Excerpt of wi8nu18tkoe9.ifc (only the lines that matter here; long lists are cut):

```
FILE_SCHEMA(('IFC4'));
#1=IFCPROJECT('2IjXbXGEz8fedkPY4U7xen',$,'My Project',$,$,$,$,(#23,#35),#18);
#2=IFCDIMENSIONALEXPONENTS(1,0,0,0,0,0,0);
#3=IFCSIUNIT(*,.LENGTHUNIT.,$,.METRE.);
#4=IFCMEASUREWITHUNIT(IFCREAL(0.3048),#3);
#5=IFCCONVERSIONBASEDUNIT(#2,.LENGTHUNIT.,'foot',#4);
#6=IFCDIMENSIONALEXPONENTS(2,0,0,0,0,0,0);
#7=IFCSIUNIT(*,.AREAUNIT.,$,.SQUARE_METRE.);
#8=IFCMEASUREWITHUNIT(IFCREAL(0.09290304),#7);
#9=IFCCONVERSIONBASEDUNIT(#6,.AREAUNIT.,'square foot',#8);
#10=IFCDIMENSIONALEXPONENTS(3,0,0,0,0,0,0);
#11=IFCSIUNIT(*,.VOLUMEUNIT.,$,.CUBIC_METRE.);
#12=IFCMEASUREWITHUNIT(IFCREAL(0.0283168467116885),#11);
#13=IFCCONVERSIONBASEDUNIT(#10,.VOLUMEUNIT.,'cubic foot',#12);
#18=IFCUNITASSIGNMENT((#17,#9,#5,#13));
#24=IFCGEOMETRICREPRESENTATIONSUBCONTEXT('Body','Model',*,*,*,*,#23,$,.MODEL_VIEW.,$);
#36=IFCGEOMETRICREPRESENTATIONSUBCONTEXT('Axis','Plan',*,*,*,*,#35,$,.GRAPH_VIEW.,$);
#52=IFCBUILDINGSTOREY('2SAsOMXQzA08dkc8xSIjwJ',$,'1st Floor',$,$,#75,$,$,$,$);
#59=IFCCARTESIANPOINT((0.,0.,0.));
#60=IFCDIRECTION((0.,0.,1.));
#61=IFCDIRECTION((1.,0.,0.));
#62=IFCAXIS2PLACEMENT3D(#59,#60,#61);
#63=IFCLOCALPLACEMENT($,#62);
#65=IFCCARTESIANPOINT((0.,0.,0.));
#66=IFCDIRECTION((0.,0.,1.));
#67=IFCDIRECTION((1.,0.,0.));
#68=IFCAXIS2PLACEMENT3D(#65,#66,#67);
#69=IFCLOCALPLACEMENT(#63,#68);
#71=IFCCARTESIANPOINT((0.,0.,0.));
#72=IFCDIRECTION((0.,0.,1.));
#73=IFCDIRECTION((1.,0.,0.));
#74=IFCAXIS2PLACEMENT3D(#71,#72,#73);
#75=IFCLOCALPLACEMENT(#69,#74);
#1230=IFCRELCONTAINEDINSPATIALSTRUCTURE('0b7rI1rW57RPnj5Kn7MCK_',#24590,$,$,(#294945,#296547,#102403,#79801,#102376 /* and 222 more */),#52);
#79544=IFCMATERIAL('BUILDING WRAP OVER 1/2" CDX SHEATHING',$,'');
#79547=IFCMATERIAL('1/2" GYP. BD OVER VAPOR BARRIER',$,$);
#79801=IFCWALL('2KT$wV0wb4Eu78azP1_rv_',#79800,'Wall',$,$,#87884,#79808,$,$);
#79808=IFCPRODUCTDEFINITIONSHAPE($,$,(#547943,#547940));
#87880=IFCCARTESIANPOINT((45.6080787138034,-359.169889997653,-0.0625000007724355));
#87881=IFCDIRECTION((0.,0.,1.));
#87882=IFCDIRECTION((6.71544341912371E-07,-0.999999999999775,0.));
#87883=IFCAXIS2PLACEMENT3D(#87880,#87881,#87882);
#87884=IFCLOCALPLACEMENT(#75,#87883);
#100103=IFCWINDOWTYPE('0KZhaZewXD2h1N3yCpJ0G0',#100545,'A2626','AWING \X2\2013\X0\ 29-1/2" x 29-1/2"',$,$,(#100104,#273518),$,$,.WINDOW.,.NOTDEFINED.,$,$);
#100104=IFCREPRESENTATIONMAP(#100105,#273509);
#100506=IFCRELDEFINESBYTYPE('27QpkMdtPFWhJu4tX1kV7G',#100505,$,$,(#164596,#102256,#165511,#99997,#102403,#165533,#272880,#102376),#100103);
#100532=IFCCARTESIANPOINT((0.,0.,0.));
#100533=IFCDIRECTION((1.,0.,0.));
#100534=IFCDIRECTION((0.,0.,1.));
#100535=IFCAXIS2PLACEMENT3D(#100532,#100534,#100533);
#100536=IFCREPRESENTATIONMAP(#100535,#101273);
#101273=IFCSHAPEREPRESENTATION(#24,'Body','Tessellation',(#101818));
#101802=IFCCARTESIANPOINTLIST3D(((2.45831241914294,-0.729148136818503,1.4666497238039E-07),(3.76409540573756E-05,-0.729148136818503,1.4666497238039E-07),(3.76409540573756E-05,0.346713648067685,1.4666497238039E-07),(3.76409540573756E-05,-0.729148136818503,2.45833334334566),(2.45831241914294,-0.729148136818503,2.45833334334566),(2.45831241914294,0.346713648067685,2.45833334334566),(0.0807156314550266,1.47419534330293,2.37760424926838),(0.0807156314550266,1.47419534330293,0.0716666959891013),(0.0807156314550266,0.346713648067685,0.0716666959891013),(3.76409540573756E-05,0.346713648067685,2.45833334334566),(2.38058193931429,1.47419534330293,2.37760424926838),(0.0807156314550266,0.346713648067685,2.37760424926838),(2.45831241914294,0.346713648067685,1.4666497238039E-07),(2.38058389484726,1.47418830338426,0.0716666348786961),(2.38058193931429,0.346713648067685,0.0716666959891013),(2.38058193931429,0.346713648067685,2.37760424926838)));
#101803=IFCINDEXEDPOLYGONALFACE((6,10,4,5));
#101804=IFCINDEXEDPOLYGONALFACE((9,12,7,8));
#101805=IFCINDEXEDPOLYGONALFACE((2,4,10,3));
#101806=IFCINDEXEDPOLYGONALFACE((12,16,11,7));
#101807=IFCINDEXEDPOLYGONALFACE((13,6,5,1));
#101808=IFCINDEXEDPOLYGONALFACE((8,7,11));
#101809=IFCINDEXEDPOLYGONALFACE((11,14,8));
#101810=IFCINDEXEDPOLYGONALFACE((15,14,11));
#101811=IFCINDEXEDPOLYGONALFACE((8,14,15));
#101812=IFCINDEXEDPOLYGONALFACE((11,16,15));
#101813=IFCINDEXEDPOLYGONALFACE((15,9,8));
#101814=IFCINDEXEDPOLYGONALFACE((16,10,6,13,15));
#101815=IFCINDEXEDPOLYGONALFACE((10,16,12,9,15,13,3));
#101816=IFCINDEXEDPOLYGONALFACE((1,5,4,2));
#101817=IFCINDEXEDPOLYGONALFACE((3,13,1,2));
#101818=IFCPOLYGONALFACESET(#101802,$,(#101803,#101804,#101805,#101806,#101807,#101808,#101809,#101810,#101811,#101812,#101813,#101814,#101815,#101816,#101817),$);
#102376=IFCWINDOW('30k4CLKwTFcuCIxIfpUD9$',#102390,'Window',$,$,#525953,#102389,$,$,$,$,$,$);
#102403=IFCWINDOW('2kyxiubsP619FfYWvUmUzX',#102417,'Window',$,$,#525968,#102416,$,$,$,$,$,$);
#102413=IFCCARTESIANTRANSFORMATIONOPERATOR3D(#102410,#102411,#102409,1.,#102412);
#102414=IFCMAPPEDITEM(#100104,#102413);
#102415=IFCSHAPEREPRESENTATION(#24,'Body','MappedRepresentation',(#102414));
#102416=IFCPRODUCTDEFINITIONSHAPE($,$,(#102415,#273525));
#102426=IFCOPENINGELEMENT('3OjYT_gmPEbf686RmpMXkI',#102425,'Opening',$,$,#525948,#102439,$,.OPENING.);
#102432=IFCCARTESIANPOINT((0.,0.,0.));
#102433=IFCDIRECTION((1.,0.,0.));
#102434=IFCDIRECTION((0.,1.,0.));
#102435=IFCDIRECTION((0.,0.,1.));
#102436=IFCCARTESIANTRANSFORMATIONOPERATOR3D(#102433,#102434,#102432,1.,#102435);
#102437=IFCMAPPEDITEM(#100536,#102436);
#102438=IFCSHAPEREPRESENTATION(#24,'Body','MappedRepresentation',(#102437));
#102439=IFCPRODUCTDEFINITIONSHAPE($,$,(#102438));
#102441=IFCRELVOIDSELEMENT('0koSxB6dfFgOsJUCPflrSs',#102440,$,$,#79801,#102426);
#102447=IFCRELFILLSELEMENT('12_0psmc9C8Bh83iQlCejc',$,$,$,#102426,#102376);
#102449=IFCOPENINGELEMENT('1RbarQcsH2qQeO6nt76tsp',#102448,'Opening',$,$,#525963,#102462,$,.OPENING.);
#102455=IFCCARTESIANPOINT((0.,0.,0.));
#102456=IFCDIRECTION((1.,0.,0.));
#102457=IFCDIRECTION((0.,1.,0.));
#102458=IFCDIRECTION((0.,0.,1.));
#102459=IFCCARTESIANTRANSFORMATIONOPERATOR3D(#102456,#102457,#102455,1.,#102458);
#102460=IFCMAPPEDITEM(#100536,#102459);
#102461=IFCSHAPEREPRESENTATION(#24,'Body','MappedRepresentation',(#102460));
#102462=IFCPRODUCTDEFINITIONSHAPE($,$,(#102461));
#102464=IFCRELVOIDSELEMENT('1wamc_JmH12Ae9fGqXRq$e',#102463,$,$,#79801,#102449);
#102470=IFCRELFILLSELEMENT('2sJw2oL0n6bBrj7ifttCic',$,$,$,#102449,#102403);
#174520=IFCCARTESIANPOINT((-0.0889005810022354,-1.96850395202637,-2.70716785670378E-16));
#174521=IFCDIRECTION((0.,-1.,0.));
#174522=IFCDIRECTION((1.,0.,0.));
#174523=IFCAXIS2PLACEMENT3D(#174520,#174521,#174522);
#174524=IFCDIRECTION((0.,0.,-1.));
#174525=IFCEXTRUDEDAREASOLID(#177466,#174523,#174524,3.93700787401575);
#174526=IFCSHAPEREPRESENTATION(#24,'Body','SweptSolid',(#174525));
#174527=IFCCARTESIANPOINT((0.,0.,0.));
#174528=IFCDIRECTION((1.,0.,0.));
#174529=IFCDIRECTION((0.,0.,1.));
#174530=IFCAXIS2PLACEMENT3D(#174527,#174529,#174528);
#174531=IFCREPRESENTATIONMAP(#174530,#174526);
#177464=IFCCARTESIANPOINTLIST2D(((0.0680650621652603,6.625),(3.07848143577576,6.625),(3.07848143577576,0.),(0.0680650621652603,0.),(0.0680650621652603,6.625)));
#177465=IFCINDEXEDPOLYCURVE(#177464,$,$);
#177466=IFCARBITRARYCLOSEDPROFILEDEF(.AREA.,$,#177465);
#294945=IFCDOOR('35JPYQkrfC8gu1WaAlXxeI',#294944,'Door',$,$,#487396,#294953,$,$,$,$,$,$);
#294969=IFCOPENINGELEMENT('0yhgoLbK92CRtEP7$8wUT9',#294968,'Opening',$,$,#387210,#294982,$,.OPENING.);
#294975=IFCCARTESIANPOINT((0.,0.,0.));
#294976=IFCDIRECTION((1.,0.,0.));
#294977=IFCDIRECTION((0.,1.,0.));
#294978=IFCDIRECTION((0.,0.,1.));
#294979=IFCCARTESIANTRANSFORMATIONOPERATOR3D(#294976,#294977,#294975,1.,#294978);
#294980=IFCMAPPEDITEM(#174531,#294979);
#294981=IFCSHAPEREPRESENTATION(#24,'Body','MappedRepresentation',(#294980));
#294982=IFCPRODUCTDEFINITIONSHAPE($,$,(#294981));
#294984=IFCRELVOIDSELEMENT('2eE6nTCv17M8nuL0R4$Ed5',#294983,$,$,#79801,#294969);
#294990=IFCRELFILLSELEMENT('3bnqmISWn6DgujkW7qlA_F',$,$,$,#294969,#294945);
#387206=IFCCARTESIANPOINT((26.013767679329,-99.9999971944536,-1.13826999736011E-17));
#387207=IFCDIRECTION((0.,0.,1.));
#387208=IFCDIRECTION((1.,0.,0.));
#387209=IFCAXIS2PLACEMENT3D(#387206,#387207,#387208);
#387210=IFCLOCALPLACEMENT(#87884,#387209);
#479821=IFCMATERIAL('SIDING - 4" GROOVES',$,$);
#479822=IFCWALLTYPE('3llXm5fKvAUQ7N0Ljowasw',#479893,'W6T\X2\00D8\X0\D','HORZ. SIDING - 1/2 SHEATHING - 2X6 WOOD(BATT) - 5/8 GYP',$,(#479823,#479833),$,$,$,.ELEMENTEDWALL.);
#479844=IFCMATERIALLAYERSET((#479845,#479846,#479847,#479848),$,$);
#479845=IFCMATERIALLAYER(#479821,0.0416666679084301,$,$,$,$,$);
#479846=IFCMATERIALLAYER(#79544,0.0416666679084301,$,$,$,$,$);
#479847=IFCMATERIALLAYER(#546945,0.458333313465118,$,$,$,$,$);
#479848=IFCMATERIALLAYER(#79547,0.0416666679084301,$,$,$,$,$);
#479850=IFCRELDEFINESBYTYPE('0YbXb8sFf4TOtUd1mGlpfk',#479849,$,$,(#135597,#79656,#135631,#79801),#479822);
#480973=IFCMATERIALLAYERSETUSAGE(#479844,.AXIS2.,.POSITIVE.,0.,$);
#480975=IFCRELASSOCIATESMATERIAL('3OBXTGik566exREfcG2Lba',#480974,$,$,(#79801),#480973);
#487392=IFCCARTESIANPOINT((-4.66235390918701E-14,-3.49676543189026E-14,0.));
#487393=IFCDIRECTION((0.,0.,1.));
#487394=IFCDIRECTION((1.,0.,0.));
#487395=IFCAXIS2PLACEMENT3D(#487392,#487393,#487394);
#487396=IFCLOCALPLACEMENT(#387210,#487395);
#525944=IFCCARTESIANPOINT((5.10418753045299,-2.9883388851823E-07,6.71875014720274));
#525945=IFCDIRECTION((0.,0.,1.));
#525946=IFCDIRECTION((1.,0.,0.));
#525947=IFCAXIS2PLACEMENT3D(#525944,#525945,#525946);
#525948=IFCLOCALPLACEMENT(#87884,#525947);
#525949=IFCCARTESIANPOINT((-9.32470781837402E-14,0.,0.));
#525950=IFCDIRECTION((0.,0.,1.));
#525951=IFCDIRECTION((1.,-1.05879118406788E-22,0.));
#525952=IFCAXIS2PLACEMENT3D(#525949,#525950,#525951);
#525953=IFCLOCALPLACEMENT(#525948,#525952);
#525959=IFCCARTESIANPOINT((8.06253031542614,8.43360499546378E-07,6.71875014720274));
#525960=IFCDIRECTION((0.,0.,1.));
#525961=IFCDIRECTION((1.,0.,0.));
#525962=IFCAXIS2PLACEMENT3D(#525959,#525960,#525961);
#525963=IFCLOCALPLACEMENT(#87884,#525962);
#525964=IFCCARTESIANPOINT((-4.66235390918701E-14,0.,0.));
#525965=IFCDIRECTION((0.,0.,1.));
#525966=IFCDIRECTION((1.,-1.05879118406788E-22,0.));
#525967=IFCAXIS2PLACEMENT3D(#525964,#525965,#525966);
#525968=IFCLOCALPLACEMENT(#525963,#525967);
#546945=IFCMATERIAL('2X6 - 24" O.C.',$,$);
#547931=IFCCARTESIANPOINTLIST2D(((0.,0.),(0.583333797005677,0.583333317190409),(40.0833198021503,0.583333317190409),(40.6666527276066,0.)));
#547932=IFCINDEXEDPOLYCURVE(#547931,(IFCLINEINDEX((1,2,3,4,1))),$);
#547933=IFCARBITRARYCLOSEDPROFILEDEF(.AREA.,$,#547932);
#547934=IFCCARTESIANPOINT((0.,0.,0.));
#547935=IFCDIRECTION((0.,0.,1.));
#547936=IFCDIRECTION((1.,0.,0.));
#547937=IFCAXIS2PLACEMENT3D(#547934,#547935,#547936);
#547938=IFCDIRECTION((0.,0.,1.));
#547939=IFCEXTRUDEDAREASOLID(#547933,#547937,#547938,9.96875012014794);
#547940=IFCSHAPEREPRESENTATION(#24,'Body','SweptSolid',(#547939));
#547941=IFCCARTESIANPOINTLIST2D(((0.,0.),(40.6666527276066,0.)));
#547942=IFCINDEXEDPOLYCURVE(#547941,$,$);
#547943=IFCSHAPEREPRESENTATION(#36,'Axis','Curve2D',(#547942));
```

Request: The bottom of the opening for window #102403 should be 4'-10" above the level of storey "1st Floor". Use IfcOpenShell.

```python
import numpy as np
import ifcopenshell
import ifcopenshell.api.geometry
import ifcopenshell.geom
import ifcopenshell.util.element
import ifcopenshell.util.placement
import ifcopenshell.util.shape
import ifcopenshell.util.unit

model = ifcopenshell.open("wi8nu18tkoe9.ifc")
unit_scale = ifcopenshell.util.unit.calculate_unit_scale(model)

window = model.by_guid("2kyxiubsP619FfYWvUmUzX")
opening = window.FillsVoids[0].RelatingOpeningElement
storey = ifcopenshell.util.element.get_container(window, ifc_class="IfcBuildingStorey")
level = ifcopenshell.util.placement.get_local_placement(storey.ObjectPlacement)[2, 3]

# The opening's origin need not be at the sill, so measure its lowest point.
shape = ifcopenshell.geom.create_shape(ifcopenshell.geom.settings(), opening)
bottom = ifcopenshell.util.shape.get_shape_bottom_elevation(shape, shape.geometry) / unit_scale
dz = level + 58 * 0.0254 / unit_scale - bottom

shift = np.array([0.0, 0.0, dz])
# The window is placed relative to its opening, so it follows when the opening moves.
matrix = ifcopenshell.util.placement.get_local_placement(opening.ObjectPlacement)
matrix[:3, 3] += shift
ifcopenshell.api.geometry.edit_object_placement(
    model, product=opening, matrix=matrix, is_si=False, should_transform_children=True
)

print(f"moved by {dz * unit_scale:+.3f} m")

model.write("wi8nu18tkoe9-out.ifc")
```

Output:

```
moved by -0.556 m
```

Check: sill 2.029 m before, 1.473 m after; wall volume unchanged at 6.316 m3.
